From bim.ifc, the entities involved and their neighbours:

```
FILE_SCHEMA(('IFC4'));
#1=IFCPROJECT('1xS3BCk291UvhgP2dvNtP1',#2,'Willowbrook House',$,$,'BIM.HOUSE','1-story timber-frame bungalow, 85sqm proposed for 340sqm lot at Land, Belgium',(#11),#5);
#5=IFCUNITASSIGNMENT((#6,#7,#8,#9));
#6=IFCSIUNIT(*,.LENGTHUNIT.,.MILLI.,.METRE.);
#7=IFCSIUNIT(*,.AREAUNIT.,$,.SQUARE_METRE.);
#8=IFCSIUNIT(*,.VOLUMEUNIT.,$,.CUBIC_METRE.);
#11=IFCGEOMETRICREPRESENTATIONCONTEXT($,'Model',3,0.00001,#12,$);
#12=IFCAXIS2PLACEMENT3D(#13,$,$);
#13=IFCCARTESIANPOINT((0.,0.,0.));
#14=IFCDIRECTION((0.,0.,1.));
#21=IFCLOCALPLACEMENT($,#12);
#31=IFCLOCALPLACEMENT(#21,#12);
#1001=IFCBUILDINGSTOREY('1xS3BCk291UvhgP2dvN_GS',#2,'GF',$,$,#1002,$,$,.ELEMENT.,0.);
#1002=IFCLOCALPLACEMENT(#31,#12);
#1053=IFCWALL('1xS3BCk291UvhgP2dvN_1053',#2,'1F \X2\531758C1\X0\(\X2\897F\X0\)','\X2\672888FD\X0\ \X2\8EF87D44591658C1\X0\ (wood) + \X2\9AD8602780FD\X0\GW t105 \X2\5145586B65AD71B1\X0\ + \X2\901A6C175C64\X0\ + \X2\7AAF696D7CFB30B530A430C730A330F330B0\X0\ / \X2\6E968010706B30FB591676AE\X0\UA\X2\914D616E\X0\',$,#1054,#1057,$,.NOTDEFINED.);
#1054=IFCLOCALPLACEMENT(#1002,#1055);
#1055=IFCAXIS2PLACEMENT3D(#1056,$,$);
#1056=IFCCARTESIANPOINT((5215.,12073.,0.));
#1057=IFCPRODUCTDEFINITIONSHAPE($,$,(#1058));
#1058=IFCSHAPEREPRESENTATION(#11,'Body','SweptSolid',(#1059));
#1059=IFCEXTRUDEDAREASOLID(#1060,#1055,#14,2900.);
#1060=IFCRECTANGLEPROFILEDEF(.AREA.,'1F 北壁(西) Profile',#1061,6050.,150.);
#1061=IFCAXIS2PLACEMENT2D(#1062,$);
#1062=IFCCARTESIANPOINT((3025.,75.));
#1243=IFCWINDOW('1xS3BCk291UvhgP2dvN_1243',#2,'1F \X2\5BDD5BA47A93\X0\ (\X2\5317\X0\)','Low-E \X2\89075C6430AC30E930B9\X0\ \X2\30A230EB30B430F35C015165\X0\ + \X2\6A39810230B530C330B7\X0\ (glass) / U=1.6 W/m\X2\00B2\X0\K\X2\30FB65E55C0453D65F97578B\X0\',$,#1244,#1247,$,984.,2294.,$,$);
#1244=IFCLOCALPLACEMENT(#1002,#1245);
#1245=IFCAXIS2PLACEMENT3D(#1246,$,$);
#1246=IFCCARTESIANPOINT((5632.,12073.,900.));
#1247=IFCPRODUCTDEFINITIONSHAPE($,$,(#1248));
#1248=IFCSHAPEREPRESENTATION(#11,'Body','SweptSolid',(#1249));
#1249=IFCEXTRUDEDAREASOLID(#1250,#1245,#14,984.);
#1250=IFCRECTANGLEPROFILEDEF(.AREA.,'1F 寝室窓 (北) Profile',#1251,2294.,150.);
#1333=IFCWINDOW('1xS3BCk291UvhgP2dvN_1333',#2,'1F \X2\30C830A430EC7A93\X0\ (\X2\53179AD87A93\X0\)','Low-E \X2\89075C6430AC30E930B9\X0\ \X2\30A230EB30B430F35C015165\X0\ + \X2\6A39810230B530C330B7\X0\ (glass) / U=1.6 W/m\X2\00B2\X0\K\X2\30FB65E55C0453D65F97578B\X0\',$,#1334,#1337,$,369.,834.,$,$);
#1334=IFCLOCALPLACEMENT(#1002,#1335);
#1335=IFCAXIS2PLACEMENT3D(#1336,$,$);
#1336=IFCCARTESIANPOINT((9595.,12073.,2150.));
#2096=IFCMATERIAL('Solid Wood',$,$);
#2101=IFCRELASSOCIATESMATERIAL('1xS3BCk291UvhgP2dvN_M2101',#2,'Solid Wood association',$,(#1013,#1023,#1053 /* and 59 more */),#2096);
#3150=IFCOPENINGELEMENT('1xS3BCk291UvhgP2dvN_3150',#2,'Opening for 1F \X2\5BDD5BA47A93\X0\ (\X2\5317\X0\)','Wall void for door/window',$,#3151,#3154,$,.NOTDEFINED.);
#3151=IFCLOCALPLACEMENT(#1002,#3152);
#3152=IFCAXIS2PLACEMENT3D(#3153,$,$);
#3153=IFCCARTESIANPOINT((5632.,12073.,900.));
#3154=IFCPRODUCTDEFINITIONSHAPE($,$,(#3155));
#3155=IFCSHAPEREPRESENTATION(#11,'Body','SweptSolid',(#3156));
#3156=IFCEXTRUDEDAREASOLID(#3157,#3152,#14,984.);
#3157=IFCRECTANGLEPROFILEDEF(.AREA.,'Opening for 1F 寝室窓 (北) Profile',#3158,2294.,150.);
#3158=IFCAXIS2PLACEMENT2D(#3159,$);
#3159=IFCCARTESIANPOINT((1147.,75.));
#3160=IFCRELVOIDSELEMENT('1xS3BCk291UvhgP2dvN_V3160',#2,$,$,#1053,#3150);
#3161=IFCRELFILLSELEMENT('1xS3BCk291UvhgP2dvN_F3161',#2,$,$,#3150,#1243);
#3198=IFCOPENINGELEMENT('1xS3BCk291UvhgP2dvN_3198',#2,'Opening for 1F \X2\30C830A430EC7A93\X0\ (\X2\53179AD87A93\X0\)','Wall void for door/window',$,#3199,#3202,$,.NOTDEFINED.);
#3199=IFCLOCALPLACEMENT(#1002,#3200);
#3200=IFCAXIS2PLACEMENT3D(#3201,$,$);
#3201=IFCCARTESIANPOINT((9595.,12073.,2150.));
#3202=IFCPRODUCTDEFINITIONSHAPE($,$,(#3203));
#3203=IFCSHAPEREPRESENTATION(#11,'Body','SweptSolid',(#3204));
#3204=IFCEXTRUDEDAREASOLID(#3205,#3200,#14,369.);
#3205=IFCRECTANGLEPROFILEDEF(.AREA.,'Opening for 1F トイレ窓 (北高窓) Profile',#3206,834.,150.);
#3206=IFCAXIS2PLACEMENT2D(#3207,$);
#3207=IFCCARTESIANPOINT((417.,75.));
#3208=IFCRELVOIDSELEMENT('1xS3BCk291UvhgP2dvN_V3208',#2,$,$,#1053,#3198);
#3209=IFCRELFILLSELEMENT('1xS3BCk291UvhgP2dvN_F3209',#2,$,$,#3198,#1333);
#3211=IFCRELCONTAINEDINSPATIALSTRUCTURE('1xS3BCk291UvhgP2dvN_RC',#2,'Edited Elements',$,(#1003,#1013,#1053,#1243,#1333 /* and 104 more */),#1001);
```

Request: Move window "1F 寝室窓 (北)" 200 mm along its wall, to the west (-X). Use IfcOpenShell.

```python
import ifcopenshell
import ifcopenshell.api.geometry
import ifcopenshell.util.placement
import ifcopenshell.util.unit

model = ifcopenshell.open("bim.ifc")
unit_scale = ifcopenshell.util.unit.calculate_unit_scale(model)

window = model.by_guid("1xS3BCk291UvhgP2dvN_1243")
opening = window.FillsVoids[0].RelatingOpeningElement
wall = opening.VoidsElements[0].RelatingBuildingElement

wall_matrix = ifcopenshell.util.placement.get_local_placement(wall.ObjectPlacement)
shift = wall_matrix[:3, 0] * -0.2 / unit_scale
before = ifcopenshell.util.placement.get_local_placement(window.ObjectPlacement)[:3, 3].copy()

# The window is not placed relative to its opening, so move both.
for product in (opening, window):
    matrix = ifcopenshell.util.placement.get_local_placement(product.ObjectPlacement)
    matrix[:3, 3] += shift
    ifcopenshell.api.geometry.edit_object_placement(model, product=product, matrix=matrix, is_si=False)

after = ifcopenshell.util.placement.get_local_placement(window.ObjectPlacement)[:3, 3]
print("window moved by", (after - before).round(3) + 0.0)

model.write("bim_edited.ifc")
```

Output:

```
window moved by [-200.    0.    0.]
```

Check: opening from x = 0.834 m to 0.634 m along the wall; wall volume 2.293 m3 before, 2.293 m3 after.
